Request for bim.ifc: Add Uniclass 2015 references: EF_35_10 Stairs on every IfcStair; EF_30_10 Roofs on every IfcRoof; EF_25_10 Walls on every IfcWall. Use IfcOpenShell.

First a look at what the model holds.

```python
import ifcopenshell

model = ifcopenshell.open("bim.ifc")
print(model.schema)
print("classifications:", [c.Name for c in model.by_type("IfcClassification")])
for ifc_class in ("IfcDoor", "IfcRoof", "IfcStair", "IfcWall", "IfcWindow"):
    print(ifc_class, len(model.by_type(ifc_class)))
```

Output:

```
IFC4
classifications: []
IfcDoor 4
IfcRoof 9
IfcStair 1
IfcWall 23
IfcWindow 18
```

```python
import ifcopenshell
import ifcopenshell.api.classification

model = ifcopenshell.open("bim.ifc")

system = ifcopenshell.api.classification.add_classification(model, classification="Uniclass 2015")

codes = {
    "IfcStair": ("EF_35_10", "Stairs"),
    "IfcRoof": ("EF_30_10", "Roofs"),
    "IfcWall": ("EF_25_10", "Walls"),
}
for ifc_class, (code, name) in codes.items():
    products = model.by_type(ifc_class)
    ifcopenshell.api.classification.add_reference(
        model, products=products, classification=system, identification=code, name=name
    )
    print(code, len(products))

model.write("bim-out.ifc")
```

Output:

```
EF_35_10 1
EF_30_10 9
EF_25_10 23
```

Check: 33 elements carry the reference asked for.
